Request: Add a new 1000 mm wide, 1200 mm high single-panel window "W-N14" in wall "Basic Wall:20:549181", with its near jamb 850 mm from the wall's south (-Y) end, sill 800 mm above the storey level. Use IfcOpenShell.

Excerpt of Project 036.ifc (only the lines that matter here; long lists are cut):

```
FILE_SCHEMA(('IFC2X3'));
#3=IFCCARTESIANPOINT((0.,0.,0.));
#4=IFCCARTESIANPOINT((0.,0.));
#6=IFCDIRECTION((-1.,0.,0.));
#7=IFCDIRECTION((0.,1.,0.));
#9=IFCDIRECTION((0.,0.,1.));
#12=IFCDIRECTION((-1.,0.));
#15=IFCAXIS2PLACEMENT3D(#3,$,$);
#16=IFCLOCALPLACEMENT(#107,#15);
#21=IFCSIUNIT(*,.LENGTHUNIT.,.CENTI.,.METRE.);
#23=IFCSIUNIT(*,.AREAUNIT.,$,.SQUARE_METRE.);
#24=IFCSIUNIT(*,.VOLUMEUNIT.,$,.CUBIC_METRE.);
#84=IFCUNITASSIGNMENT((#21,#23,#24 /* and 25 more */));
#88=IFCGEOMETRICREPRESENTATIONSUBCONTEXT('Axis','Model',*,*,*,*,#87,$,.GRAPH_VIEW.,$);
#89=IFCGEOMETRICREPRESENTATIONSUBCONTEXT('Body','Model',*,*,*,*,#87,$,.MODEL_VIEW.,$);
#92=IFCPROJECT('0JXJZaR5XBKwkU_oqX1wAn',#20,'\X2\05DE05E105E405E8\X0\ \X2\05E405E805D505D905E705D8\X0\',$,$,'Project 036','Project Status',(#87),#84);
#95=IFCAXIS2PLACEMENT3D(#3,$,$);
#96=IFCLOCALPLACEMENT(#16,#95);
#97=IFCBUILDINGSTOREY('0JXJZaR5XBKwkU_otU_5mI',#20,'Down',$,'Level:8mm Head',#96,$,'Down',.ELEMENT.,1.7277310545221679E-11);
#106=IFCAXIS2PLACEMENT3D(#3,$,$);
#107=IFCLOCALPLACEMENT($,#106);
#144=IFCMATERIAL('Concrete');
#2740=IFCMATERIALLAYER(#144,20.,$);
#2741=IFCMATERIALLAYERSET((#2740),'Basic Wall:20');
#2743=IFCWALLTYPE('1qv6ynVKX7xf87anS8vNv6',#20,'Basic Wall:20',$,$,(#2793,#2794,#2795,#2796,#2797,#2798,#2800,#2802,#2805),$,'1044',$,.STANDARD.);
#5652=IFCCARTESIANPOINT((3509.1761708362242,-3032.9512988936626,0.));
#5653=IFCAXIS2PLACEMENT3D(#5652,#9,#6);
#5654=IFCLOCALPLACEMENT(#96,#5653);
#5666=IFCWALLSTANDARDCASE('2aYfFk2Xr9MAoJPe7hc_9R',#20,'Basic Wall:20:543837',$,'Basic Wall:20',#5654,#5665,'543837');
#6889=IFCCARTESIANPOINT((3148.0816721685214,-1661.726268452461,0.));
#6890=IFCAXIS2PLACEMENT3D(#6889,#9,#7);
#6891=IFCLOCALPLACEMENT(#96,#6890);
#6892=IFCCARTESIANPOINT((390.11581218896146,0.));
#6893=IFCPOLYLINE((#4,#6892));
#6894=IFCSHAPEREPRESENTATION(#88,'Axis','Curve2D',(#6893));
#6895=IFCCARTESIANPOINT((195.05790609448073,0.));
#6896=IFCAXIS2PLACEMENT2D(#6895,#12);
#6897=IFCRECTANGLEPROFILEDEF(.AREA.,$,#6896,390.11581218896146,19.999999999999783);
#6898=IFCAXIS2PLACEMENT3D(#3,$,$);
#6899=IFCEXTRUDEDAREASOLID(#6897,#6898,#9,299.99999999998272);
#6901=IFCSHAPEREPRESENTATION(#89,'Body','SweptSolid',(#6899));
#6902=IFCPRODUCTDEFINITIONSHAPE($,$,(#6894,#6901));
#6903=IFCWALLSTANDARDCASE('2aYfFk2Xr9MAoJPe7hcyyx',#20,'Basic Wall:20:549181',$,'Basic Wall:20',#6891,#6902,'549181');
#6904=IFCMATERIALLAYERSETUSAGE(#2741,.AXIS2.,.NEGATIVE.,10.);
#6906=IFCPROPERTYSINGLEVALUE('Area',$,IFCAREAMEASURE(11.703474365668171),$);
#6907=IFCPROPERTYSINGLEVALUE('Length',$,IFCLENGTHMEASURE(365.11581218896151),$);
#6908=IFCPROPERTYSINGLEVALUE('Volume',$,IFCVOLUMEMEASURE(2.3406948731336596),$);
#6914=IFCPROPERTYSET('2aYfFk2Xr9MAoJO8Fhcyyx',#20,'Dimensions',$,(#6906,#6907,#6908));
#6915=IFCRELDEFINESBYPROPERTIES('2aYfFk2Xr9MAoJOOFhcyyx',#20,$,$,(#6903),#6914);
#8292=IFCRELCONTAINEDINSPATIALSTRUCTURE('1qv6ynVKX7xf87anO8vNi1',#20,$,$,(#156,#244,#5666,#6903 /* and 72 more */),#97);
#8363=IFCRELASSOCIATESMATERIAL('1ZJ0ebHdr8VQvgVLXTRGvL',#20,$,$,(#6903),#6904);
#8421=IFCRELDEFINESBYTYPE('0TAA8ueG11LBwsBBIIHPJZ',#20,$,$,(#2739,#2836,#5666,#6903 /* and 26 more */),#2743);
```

```python
import numpy as np
import ifcopenshell
import ifcopenshell.api.feature
import ifcopenshell.api.geometry
import ifcopenshell.api.pset
import ifcopenshell.api.root
import ifcopenshell.api.spatial
import ifcopenshell.api.type
import ifcopenshell.geom
import ifcopenshell.util.element
import ifcopenshell.util.placement
import ifcopenshell.util.representation
import ifcopenshell.util.shape
import ifcopenshell.util.unit

model = ifcopenshell.open("Project 036.ifc")
unit_scale = ifcopenshell.util.unit.calculate_unit_scale(model)
area_scale = ifcopenshell.util.unit.calculate_unit_scale(model, "AREAUNIT")
volume_scale = ifcopenshell.util.unit.calculate_unit_scale(model, "VOLUMEUNIT")
settings = ifcopenshell.geom.settings()


def volume(element):
    """Net volume in cubic metres, openings subtracted."""
    shape = ifcopenshell.geom.create_shape(settings, element)
    return ifcopenshell.util.shape.get_volume(shape.geometry)


wall = model.by_guid("2aYfFk2Xr9MAoJPe7hcyyx")
storey = ifcopenshell.util.element.get_container(wall, ifc_class="IfcBuildingStorey")
context = ifcopenshell.util.representation.get_context(model, "Model", "Body", "MODEL_VIEW")
before = volume(wall)

width, height, from_end, sill = 1, 1.2, 0.85, 0.8  # metres

# The wall runs along its own X axis, and the end named is its -X end.
wall_shape = ifcopenshell.geom.create_shape(settings, wall)
x, y, z = ifcopenshell.util.shape.get_vertices(wall_shape.geometry).T
start = x.min() + from_end
face, thickness = float(y.min()), float(y.max() - y.min())
wall_matrix = ifcopenshell.util.placement.get_local_placement(wall.ObjectPlacement)
level = ifcopenshell.util.placement.get_local_placement(storey.ObjectPlacement)[2, 3]


def in_wall(x, y):
    """Placement at x, y metres in the wall's axes, at sill height."""
    matrix = wall_matrix.copy()
    matrix[:, 3] = wall_matrix @ np.array([x / unit_scale, y / unit_scale, 0.0, 1.0])
    matrix[2, 3] = level + sill / unit_scale
    return matrix


# Opening: a box that overshoots both wall faces by 50 mm.
opening = ifcopenshell.api.root.create_entity(model, ifc_class="IfcOpeningElement")
box = ifcopenshell.api.geometry.add_wall_representation(
    model, context=context, length=width, height=height, thickness=thickness + 0.1
)
ifcopenshell.api.geometry.assign_representation(model, product=opening, representation=box)
ifcopenshell.api.geometry.edit_object_placement(model, product=opening, matrix=in_wall(start, face - 0.05), is_si=False)
ifcopenshell.api.feature.add_feature(model, feature=opening, element=wall)

window = ifcopenshell.api.root.create_entity(model, ifc_class="IfcWindow", name="W-N14")
window.OverallWidth, window.OverallHeight = width / unit_scale, height / unit_scale
body = ifcopenshell.api.geometry.add_window_representation(
    model,
    context=context,
    overall_width=window.OverallWidth,
    overall_height=window.OverallHeight,
    partition_type="SINGLE_PANEL",
)
ifcopenshell.api.geometry.assign_representation(model, product=window, representation=body)
ifcopenshell.api.spatial.assign_container(model, products=[window], relating_structure=storey)
fills = ifcopenshell.api.feature.add_filling(model, opening=opening, element=window)
fills.OwnerHistory = window.OwnerHistory  # required in IFC2X3

# IFC2X3 keeps the operation on the window style.
style = ifcopenshell.api.root.create_entity(model, ifc_class="IfcWindowStyle", name="W-N14")
style.OperationType, style.ConstructionType = "SINGLE_PANEL", "NOTDEFINED"
style.ParameterTakesPrecedence = style.Sizeable = False
ifcopenshell.api.type.assign_type(model, related_objects=[window], relating_type=style)

# Centre the window in the wall's thickness.
ifcopenshell.api.geometry.edit_object_placement(model, product=window, matrix=in_wall(start, face), is_si=False)
window_shape = ifcopenshell.geom.create_shape(settings, window)
depth = ifcopenshell.util.shape.get_vertices(window_shape.geometry)[:, 1]
offset = face + thickness / 2 - (depth.min() + depth.max()) / 2
ifcopenshell.api.geometry.edit_object_placement(model, product=window, matrix=in_wall(start, offset), is_si=False)

after = volume(wall)

# Update the wall's stored quantities.
pset = model.by_id(ifcopenshell.util.element.get_pset(wall, "Dimensions", should_inherit=False)["id"])
ifcopenshell.api.pset.edit_pset(model, pset=pset, properties={
    "Area": model.create_entity("IfcAreaMeasure", after / thickness / area_scale),
    "Volume": model.create_entity("IfcVolumeMeasure", after / volume_scale),
})

print(f"wall volume {before:.3f} -> {after:.3f} m3")

model.write("Project 036-out.ifc")
```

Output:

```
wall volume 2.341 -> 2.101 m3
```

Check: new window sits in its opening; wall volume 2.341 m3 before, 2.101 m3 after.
